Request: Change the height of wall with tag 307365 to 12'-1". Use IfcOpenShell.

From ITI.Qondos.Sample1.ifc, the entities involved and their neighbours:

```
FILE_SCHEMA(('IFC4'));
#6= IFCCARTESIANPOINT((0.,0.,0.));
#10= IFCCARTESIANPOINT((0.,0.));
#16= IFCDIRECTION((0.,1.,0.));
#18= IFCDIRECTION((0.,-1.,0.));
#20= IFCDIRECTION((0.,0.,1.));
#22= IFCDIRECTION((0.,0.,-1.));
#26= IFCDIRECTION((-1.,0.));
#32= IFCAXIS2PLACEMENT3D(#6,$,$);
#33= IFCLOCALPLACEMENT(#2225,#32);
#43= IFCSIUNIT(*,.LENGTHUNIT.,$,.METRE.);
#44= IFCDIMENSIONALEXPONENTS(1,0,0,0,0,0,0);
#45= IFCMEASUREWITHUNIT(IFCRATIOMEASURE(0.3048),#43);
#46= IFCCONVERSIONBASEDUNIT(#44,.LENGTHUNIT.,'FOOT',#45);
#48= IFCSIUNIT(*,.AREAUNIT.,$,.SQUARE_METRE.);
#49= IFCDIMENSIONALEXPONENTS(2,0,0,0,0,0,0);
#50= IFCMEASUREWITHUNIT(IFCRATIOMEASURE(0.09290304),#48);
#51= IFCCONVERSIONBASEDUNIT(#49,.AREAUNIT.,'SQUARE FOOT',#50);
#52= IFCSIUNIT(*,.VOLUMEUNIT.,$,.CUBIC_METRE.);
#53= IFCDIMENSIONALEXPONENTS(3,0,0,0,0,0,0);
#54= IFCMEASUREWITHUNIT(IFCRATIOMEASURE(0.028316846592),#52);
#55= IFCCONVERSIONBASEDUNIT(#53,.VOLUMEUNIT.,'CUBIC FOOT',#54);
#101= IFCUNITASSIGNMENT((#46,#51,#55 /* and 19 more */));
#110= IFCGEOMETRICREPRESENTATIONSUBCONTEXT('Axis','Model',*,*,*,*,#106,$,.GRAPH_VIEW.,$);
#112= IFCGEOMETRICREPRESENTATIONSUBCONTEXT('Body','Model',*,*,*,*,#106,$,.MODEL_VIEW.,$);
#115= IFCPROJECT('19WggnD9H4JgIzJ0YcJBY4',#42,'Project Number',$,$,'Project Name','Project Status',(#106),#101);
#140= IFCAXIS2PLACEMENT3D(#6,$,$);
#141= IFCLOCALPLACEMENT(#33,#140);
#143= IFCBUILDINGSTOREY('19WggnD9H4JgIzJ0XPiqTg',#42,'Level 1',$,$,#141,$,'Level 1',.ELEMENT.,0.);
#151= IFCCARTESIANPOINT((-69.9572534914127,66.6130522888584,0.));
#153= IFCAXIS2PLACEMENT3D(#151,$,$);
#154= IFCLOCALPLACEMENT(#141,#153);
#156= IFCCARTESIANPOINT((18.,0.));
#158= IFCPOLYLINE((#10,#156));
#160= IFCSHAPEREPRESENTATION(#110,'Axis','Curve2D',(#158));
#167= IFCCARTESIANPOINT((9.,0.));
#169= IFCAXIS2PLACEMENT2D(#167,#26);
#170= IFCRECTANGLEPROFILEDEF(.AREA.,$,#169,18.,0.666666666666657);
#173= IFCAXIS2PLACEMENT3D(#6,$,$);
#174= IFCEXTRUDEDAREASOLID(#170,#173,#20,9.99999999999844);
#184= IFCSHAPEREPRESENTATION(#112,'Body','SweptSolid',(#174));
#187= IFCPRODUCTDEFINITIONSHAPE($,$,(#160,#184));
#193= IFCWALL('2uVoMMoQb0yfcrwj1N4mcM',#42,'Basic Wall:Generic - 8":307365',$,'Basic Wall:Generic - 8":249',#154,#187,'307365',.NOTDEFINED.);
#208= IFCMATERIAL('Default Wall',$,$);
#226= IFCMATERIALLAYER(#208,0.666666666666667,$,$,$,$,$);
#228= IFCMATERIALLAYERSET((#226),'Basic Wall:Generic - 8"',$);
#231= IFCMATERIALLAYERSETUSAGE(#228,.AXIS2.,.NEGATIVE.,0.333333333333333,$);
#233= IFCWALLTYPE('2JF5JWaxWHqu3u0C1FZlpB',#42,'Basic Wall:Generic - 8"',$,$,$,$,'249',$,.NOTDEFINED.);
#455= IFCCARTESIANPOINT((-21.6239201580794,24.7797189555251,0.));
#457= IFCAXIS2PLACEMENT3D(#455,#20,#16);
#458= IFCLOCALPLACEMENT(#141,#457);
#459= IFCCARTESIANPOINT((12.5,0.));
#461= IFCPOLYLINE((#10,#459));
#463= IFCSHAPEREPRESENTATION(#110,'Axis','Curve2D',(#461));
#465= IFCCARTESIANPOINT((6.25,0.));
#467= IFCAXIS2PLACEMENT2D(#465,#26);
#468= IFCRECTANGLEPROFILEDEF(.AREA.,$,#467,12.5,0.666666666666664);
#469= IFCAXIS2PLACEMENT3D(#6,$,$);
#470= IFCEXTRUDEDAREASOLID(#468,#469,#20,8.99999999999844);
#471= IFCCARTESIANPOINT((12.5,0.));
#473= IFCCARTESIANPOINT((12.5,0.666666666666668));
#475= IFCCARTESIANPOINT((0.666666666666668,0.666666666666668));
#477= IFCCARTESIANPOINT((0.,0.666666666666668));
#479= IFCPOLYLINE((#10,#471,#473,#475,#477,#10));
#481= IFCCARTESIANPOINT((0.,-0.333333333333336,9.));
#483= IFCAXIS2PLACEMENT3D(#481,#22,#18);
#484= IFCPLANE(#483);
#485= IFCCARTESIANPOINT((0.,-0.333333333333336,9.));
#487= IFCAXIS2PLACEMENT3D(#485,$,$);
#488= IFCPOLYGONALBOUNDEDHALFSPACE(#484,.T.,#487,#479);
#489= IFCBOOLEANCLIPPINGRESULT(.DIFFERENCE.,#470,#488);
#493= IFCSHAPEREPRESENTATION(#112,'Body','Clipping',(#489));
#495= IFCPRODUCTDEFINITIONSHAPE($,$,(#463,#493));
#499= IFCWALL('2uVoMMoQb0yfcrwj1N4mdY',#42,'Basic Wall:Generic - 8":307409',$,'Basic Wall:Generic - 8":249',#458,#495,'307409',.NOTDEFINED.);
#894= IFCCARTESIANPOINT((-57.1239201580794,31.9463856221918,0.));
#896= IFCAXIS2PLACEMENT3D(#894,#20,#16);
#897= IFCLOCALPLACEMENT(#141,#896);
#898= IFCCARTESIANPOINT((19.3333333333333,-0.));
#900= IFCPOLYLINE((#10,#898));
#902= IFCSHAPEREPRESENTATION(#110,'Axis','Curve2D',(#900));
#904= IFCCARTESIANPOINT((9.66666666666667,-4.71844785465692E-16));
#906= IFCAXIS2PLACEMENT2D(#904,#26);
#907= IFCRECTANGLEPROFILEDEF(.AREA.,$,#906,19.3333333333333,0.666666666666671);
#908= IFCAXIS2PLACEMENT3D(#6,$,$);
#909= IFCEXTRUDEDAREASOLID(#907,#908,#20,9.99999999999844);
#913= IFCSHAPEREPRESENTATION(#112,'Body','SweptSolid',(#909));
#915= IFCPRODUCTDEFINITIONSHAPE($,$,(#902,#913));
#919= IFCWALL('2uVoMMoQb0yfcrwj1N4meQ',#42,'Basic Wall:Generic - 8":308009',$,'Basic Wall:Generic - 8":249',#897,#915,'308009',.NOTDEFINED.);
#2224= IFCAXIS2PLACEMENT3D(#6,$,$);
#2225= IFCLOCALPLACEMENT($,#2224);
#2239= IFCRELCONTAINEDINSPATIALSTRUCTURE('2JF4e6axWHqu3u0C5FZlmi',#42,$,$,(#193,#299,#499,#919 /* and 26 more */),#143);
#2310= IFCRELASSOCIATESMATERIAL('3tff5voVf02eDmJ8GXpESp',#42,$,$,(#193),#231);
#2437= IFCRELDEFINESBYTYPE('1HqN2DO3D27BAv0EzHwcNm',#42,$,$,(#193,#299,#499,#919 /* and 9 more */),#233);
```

```python
import ifcopenshell
import ifcopenshell.geom
import ifcopenshell.util.representation
import ifcopenshell.util.shape
import ifcopenshell.util.unit

model = ifcopenshell.open("ITI.Qondos.Sample1.ifc")
unit_scale = ifcopenshell.util.unit.calculate_unit_scale(model)
settings = ifcopenshell.geom.settings()


def volume(element):
    """Net volume in cubic metres, openings subtracted."""
    shape = ifcopenshell.geom.create_shape(settings, element)
    return ifcopenshell.util.shape.get_volume(shape.geometry)


wall = model.by_id(193)
before = volume(wall)

body = ifcopenshell.util.representation.get_representation(wall, "Model", "Body")
solid = body.Items[0]
old_height = solid.Depth
solid.Depth = 145 * 0.0254 / unit_scale
after = volume(wall)

print(f"height {old_height:g} -> {solid.Depth:g}, volume {before:.3f} -> {after:.3f} m3")

model.write("ITI.Qondos.Sample1_edited.ifc")
```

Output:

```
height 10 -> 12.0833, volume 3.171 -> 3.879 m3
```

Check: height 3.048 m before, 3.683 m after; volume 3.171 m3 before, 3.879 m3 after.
